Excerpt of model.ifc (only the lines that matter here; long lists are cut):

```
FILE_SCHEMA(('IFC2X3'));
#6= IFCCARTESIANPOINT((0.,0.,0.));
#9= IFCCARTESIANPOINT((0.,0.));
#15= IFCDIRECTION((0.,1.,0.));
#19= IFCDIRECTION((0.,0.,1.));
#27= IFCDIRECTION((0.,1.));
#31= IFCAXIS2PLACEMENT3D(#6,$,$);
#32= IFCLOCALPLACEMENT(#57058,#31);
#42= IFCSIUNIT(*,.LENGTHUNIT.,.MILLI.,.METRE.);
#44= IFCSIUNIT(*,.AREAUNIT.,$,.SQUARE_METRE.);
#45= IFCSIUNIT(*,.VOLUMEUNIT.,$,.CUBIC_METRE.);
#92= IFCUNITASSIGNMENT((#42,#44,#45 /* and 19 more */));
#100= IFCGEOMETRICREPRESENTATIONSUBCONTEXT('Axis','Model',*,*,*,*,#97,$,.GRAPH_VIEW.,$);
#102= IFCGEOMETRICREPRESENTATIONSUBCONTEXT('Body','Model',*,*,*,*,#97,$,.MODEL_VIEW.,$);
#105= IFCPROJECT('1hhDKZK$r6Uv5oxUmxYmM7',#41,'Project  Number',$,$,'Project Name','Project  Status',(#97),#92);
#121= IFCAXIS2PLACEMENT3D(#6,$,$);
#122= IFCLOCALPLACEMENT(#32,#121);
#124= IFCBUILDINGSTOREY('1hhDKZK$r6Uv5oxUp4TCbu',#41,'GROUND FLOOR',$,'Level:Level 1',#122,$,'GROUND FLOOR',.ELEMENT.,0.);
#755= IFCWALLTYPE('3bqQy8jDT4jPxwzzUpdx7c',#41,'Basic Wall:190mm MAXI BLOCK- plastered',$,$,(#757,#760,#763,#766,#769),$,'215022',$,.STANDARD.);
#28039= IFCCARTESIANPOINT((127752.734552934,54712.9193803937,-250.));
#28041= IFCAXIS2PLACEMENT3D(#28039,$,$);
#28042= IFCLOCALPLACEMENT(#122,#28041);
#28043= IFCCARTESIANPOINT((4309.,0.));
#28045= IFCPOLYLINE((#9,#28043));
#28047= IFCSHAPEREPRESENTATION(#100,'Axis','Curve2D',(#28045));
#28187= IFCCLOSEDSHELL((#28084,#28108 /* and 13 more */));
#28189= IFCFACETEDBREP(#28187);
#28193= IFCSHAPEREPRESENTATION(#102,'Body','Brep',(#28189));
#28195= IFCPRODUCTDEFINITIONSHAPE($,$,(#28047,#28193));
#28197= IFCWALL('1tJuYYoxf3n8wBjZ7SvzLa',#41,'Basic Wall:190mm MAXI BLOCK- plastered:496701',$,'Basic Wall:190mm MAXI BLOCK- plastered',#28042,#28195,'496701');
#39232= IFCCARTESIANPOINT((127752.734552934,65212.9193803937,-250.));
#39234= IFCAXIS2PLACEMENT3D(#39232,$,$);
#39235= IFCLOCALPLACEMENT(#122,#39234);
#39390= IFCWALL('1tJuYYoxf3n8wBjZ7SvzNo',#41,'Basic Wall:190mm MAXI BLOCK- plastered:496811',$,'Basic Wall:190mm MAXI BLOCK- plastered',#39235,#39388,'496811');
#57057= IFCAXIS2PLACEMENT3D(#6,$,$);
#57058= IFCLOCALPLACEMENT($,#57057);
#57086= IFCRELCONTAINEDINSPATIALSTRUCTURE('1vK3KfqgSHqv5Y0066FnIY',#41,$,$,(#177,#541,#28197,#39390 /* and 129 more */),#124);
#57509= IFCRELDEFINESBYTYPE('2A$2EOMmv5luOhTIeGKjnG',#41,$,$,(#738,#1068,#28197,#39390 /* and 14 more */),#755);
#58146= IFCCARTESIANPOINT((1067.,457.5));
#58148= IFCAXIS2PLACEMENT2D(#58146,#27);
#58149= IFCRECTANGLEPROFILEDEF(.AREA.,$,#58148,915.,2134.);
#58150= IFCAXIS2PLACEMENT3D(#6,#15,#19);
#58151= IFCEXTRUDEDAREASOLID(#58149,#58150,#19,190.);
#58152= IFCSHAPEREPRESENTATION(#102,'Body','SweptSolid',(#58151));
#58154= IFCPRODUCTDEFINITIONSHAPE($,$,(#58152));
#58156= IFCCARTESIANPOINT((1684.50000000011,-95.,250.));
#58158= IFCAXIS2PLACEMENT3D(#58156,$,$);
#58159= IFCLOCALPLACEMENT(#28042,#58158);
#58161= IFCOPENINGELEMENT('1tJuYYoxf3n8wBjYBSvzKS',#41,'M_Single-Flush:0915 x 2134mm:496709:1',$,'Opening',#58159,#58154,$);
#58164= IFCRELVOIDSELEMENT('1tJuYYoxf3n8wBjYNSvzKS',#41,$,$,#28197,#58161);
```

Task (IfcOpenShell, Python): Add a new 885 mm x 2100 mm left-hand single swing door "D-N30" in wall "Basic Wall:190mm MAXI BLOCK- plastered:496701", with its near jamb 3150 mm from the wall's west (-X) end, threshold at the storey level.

```python
import numpy as np
import ifcopenshell
import ifcopenshell.api.feature
import ifcopenshell.api.geometry
import ifcopenshell.api.root
import ifcopenshell.api.spatial
import ifcopenshell.api.type
import ifcopenshell.geom
import ifcopenshell.util.element
import ifcopenshell.util.placement
import ifcopenshell.util.representation
import ifcopenshell.util.shape
import ifcopenshell.util.unit

model = ifcopenshell.open("model.ifc")
unit_scale = ifcopenshell.util.unit.calculate_unit_scale(model)
settings = ifcopenshell.geom.settings()


def volume(element):
    """Net volume in cubic metres, openings subtracted."""
    shape = ifcopenshell.geom.create_shape(settings, element)
    return ifcopenshell.util.shape.get_volume(shape.geometry)


wall = model.by_guid("1tJuYYoxf3n8wBjZ7SvzLa")
storey = ifcopenshell.util.element.get_container(wall, ifc_class="IfcBuildingStorey")
context = ifcopenshell.util.representation.get_context(model, "Model", "Body", "MODEL_VIEW")
before = volume(wall)

width, height, from_end, sill = 0.885, 2.1, 3.15, 0.0  # metres

# The wall runs along its own X axis, and the end named is its -X end.
wall_shape = ifcopenshell.geom.create_shape(settings, wall)
x, y, z = ifcopenshell.util.shape.get_vertices(wall_shape.geometry).T
start = x.min() + from_end
face, thickness = float(y.min()), float(y.max() - y.min())
wall_matrix = ifcopenshell.util.placement.get_local_placement(wall.ObjectPlacement)
level = ifcopenshell.util.placement.get_local_placement(storey.ObjectPlacement)[2, 3]


def in_wall(x, y):
    """Placement at x, y metres in the wall's axes, at sill height."""
    matrix = wall_matrix.copy()
    matrix[:, 3] = wall_matrix @ np.array([x / unit_scale, y / unit_scale, 0.0, 1.0])
    matrix[2, 3] = level + sill / unit_scale
    return matrix


# Opening: a box that overshoots both wall faces by 50 mm.
opening = ifcopenshell.api.root.create_entity(model, ifc_class="IfcOpeningElement")
box = ifcopenshell.api.geometry.add_wall_representation(
    model, context=context, length=width, height=height, thickness=thickness + 0.1
)
ifcopenshell.api.geometry.assign_representation(model, product=opening, representation=box)
ifcopenshell.api.geometry.edit_object_placement(model, product=opening, matrix=in_wall(start, face - 0.05), is_si=False)
ifcopenshell.api.feature.add_feature(model, feature=opening, element=wall)

door = ifcopenshell.api.root.create_entity(model, ifc_class="IfcDoor", name="D-N30")
door.OverallWidth, door.OverallHeight = width / unit_scale, height / unit_scale
body = ifcopenshell.api.geometry.add_door_representation(
    model,
    context=context,
    overall_width=door.OverallWidth,
    overall_height=door.OverallHeight,
    operation_type="SINGLE_SWING_LEFT",
    lining_properties={"LiningDepth": thickness / unit_scale, "ThresholdDepth": thickness / unit_scale},
)
ifcopenshell.api.geometry.assign_representation(model, product=door, representation=body)
ifcopenshell.api.spatial.assign_container(model, products=[door], relating_structure=storey)
fills = ifcopenshell.api.feature.add_filling(model, opening=opening, element=door)
fills.OwnerHistory = door.OwnerHistory  # required in IFC2X3

# IFC2X3 keeps the operation on the door style.
style = ifcopenshell.api.root.create_entity(model, ifc_class="IfcDoorStyle", name="D-N30")
style.OperationType, style.ConstructionType = "SINGLE_SWING_LEFT", "NOTDEFINED"
style.ParameterTakesPrecedence = style.Sizeable = False
ifcopenshell.api.type.assign_type(model, related_objects=[door], relating_type=style)

# The lining spans the wall, so the door starts at the wall face.
ifcopenshell.api.geometry.edit_object_placement(model, product=door, matrix=in_wall(start, face), is_si=False)

after = volume(wall)

print(f"wall volume {before:.3f} -> {after:.3f} m3")

model.write("model_updated.ifc")
```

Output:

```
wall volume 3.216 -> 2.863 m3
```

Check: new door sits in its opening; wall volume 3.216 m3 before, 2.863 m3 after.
